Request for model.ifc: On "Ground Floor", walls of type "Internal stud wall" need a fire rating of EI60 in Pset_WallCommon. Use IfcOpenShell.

First a look at what the model holds.

```python
import ifcopenshell
import ifcopenshell.util.element

model = ifcopenshell.open("model.ifc")
print(model.schema)
storey = next(s for s in model.by_type("IfcBuildingStorey") if s.Name == "Ground Floor")
walls = [e for e in ifcopenshell.util.element.get_decomposition(storey) if e.is_a("IfcWall")]
seen = {}
for e in walls:
    element_type = ifcopenshell.util.element.get_type(e)
    key = (element_type.Name if element_type != e and element_type else None, ifcopenshell.util.element.get_pset(e, "Pset_WallCommon", "FireRating"))
    seen[key] = seen.get(key, 0) + 1
for (name, value), count in sorted(seen.items(), key=str):
    print(count, "x", name, "|", value)
```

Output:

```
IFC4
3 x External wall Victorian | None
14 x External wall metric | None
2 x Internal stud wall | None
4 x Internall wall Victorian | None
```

```python
import ifcopenshell
import ifcopenshell.api.pset
import ifcopenshell.util.element

model = ifcopenshell.open("model.ifc")

storey = next(s for s in model.by_type("IfcBuildingStorey") if s.Name == "Ground Floor")
walls = [e for e in ifcopenshell.util.element.get_decomposition(storey) if e.is_a("IfcWall")]

count = 0
for e in walls:
    element_type = ifcopenshell.util.element.get_type(e)
    if element_type in (None, e) or element_type.Name != "Internal stud wall":
        continue
    # add_pset returns the element's existing set when there is one.
    pset = ifcopenshell.api.pset.add_pset(model, product=e, name="Pset_WallCommon")
    ifcopenshell.api.pset.edit_pset(model, pset=pset, properties={"FireRating": "EI60"})
    count += 1

print(count, "walls updated")

model.write("model_v2.ifc")
```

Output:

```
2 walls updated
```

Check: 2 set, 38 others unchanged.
